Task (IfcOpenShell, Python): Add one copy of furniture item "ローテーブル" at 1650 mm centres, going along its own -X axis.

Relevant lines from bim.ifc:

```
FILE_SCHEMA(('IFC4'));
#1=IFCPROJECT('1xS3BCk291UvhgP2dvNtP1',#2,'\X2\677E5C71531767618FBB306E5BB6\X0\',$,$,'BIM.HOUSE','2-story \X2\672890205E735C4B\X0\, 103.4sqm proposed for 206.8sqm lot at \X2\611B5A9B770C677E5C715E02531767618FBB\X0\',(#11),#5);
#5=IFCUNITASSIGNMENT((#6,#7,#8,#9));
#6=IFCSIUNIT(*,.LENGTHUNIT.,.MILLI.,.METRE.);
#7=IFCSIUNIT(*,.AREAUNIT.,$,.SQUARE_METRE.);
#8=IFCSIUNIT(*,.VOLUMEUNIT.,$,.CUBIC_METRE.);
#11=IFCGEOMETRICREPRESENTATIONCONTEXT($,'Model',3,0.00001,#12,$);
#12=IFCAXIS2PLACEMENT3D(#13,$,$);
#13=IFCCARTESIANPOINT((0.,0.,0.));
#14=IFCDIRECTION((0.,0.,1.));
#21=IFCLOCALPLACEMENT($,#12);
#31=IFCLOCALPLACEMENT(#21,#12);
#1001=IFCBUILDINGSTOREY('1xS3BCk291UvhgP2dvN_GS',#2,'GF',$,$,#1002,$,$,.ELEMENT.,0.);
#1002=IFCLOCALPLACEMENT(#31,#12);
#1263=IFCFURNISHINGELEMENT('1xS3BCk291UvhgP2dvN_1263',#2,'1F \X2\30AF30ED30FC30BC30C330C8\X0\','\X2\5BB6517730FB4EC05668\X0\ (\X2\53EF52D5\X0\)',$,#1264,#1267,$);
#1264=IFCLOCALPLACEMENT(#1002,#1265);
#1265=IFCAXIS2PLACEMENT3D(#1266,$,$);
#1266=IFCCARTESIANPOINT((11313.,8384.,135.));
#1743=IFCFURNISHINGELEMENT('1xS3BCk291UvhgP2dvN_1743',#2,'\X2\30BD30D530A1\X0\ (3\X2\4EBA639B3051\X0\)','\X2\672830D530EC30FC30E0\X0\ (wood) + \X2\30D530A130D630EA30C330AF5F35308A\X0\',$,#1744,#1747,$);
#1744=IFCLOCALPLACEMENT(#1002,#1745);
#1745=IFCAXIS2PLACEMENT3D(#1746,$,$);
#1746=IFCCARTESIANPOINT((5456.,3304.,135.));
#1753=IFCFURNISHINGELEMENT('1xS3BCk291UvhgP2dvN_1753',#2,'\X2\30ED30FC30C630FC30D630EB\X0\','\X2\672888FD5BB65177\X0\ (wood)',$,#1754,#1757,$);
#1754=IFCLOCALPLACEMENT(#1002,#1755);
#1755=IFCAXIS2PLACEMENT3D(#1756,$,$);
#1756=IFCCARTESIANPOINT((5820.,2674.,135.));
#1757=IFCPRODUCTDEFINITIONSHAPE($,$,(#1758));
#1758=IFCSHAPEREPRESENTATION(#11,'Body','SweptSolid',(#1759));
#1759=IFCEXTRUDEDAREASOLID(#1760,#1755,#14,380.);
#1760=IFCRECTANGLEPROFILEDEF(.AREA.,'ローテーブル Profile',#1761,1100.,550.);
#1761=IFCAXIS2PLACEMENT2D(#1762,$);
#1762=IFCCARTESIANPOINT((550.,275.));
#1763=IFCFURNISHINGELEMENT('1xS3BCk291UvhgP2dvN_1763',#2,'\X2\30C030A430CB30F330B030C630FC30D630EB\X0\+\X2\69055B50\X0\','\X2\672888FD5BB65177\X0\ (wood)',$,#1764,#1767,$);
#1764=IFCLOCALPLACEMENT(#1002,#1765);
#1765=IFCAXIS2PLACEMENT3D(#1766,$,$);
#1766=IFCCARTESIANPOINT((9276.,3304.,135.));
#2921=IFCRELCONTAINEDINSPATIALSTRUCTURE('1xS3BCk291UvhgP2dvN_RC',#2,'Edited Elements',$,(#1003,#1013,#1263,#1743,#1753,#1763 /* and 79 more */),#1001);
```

```python
import ifcopenshell
import ifcopenshell.api.geometry
import ifcopenshell.api.root
import ifcopenshell.util.element
import ifcopenshell.util.placement

model = ifcopenshell.open("bim.ifc")


def reuse_history(source, copy):
    """copy_class also copies each property set's owner history, people and application; keep the originals."""
    for rel in copy.IsDefinedBy:
        if rel.is_a("IfcRelDefinesByProperties") and (history := rel.RelatingPropertyDefinition.OwnerHistory):
            rel.RelatingPropertyDefinition.OwnerHistory = source.OwnerHistory
            ifcopenshell.util.element.remove_deep2(model, history)


source = model.by_guid("1xS3BCk291UvhgP2dvN_1753")
base = ifcopenshell.util.placement.get_local_placement(source.ObjectPlacement)
step = -base[:3, 0] * 1650.0

for i in range(1, 2):
    copy = ifcopenshell.api.root.copy_class(model, product=source)
    copy.Representation = ifcopenshell.util.element.copy_deep(
        model, source.Representation, exclude=["IfcGeometricRepresentationContext", "IfcRepresentationMap"]
    )
    reuse_history(source, copy)
    matrix = base.copy()
    matrix[:3, 3] += i * step
    print("added at", matrix[:3, 3].round(3) + 0.0)
    ifcopenshell.api.geometry.edit_object_placement(model, product=copy, matrix=matrix, is_si=False)

model.write("bim_rev.ifc")
```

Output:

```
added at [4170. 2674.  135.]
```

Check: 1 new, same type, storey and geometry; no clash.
